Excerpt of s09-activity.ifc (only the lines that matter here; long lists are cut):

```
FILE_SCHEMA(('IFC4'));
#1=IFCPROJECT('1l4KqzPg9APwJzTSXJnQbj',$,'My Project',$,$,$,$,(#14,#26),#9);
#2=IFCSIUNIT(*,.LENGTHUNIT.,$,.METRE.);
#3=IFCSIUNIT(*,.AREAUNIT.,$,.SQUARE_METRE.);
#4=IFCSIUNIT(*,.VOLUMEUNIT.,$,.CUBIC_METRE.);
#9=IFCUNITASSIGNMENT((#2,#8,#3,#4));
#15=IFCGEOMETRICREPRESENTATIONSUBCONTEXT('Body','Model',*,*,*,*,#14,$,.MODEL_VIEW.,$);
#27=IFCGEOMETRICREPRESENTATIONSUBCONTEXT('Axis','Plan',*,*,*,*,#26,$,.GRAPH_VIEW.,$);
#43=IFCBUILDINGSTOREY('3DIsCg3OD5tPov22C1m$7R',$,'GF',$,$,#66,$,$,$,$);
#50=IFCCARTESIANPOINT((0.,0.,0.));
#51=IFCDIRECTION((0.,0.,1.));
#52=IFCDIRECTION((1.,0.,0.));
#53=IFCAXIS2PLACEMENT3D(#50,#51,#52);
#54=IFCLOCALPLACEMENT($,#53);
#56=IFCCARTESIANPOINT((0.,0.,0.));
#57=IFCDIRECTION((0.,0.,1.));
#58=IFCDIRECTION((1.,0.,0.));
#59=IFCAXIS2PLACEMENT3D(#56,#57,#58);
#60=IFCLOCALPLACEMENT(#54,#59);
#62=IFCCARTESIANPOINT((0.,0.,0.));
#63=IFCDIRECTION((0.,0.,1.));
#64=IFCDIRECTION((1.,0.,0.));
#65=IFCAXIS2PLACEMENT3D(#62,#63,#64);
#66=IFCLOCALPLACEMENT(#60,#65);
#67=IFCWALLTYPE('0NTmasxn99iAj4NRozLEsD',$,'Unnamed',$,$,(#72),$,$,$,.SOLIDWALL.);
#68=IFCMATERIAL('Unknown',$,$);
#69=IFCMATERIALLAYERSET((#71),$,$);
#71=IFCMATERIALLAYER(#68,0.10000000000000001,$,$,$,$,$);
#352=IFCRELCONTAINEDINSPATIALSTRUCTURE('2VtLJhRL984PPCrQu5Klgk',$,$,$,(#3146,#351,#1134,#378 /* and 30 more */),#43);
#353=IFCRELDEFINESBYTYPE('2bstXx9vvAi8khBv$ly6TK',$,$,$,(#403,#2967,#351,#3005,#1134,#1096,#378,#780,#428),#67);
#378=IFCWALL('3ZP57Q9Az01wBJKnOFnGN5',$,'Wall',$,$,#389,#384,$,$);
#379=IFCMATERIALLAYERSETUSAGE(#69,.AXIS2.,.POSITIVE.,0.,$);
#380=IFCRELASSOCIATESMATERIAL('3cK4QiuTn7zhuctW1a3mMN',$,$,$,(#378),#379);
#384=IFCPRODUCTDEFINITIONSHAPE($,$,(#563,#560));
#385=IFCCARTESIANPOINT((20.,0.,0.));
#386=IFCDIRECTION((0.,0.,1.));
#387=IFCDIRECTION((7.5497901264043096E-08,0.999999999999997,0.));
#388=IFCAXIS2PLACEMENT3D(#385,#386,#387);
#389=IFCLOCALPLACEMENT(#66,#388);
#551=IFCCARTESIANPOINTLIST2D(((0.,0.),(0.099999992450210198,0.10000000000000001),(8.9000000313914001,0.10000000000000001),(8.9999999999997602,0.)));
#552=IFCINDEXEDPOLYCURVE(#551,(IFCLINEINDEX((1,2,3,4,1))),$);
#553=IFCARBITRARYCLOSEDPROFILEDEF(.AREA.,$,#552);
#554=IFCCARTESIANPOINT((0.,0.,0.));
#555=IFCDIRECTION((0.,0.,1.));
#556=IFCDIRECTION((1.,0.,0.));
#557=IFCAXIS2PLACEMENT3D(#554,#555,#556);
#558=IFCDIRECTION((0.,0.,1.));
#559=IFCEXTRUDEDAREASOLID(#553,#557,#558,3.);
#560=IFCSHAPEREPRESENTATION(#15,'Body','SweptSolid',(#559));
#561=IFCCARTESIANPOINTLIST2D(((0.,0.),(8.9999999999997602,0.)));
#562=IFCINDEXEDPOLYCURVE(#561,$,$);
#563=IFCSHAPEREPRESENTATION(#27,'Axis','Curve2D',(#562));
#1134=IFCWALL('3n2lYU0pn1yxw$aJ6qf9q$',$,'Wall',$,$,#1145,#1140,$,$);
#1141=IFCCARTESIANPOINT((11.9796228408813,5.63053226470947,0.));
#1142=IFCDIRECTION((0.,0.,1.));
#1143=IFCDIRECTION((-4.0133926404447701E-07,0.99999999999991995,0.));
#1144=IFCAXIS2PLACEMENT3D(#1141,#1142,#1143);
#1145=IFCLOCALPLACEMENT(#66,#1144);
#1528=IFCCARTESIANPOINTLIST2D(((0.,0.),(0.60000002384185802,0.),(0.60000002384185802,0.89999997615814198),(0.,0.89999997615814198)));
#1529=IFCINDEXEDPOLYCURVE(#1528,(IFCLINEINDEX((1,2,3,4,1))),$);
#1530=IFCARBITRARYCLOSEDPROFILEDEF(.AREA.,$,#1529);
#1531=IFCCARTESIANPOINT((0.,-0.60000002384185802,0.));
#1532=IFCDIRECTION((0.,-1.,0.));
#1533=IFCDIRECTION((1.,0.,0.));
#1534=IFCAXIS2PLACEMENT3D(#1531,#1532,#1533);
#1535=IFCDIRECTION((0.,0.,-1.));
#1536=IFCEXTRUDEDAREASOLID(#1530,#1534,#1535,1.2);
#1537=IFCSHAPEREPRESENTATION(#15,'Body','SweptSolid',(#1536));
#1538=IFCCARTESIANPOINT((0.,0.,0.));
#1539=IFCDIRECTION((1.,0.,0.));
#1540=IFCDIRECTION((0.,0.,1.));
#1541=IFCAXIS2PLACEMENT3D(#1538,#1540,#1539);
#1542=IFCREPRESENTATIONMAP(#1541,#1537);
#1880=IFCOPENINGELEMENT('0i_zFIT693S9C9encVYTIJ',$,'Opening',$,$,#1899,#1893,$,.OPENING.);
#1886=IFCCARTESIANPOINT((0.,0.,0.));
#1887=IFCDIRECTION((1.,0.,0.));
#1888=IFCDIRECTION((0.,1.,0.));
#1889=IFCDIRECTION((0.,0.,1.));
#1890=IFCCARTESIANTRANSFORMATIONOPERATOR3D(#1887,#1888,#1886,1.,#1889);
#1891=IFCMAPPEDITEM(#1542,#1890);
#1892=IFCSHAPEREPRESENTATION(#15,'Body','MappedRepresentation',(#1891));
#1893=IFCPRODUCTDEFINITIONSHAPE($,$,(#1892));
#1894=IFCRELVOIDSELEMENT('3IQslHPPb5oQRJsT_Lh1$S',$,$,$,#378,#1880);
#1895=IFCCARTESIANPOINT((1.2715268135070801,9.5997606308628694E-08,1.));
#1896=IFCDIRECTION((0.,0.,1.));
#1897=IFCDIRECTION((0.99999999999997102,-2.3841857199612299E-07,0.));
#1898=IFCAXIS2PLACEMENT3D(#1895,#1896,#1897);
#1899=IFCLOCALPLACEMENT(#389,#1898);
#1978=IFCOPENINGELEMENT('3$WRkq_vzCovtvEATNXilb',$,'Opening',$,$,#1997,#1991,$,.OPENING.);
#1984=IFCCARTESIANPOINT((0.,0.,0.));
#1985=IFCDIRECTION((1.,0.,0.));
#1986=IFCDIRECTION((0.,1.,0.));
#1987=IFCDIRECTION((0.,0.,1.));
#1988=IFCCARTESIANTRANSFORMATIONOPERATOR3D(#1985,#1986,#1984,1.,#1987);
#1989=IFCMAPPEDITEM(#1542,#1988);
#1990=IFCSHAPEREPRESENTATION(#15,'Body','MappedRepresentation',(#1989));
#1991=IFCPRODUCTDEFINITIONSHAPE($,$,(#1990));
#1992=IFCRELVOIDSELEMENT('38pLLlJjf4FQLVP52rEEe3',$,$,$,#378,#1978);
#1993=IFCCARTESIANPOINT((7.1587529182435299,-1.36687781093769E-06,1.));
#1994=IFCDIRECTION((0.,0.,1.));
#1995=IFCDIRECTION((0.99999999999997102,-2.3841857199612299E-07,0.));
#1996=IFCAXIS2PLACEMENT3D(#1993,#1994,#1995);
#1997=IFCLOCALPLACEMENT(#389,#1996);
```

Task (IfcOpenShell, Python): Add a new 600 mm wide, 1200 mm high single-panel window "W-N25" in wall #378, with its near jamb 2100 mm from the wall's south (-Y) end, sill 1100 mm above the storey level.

```python
import numpy as np
import ifcopenshell
import ifcopenshell.api.feature
import ifcopenshell.api.geometry
import ifcopenshell.api.root
import ifcopenshell.api.spatial
import ifcopenshell.geom
import ifcopenshell.util.element
import ifcopenshell.util.placement
import ifcopenshell.util.representation
import ifcopenshell.util.shape
import ifcopenshell.util.unit

model = ifcopenshell.open("s09-activity.ifc")
unit_scale = ifcopenshell.util.unit.calculate_unit_scale(model)
settings = ifcopenshell.geom.settings()


def volume(element):
    """Net volume in cubic metres, openings subtracted."""
    shape = ifcopenshell.geom.create_shape(settings, element)
    return ifcopenshell.util.shape.get_volume(shape.geometry)


wall = model.by_guid("3ZP57Q9Az01wBJKnOFnGN5")
storey = ifcopenshell.util.element.get_container(wall, ifc_class="IfcBuildingStorey")
context = ifcopenshell.util.representation.get_context(model, "Model", "Body", "MODEL_VIEW")
before = volume(wall)

width, height, from_end, sill = 0.6, 1.2, 2.1, 1.1  # metres

# The wall runs along its own X axis, and the end named is its -X end.
wall_shape = ifcopenshell.geom.create_shape(settings, wall)
x, y, z = ifcopenshell.util.shape.get_vertices(wall_shape.geometry).T
start = x.min() + from_end
face, thickness = float(y.min()), float(y.max() - y.min())
wall_matrix = ifcopenshell.util.placement.get_local_placement(wall.ObjectPlacement)
level = ifcopenshell.util.placement.get_local_placement(storey.ObjectPlacement)[2, 3]


def in_wall(x, y):
    """Placement at x, y metres in the wall's axes, at sill height."""
    matrix = wall_matrix.copy()
    matrix[:, 3] = wall_matrix @ np.array([x / unit_scale, y / unit_scale, 0.0, 1.0])
    matrix[2, 3] = level + sill / unit_scale
    return matrix


# Opening: a box that overshoots both wall faces by 50 mm.
opening = ifcopenshell.api.root.create_entity(model, ifc_class="IfcOpeningElement", predefined_type="OPENING")
box = ifcopenshell.api.geometry.add_wall_representation(
    model, context=context, length=width, height=height, thickness=thickness + 0.1
)
ifcopenshell.api.geometry.assign_representation(model, product=opening, representation=box)
ifcopenshell.api.geometry.edit_object_placement(model, product=opening, matrix=in_wall(start, face - 0.05), is_si=False)
ifcopenshell.api.feature.add_feature(model, feature=opening, element=wall)

window = ifcopenshell.api.root.create_entity(model, ifc_class="IfcWindow", name="W-N25", predefined_type="WINDOW")
window.OverallWidth, window.OverallHeight = width / unit_scale, height / unit_scale
window.PartitioningType = "SINGLE_PANEL"
body = ifcopenshell.api.geometry.add_window_representation(
    model,
    context=context,
    overall_width=window.OverallWidth,
    overall_height=window.OverallHeight,
    partition_type="SINGLE_PANEL",
)
ifcopenshell.api.geometry.assign_representation(model, product=window, representation=body)
ifcopenshell.api.spatial.assign_container(model, products=[window], relating_structure=storey)
ifcopenshell.api.feature.add_filling(model, opening=opening, element=window)

# Centre the window in the wall's thickness.
ifcopenshell.api.geometry.edit_object_placement(model, product=window, matrix=in_wall(start, face), is_si=False)
window_shape = ifcopenshell.geom.create_shape(settings, window)
depth = ifcopenshell.util.shape.get_vertices(window_shape.geometry)[:, 1]
offset = face + thickness / 2 - (depth.min() + depth.max()) / 2
ifcopenshell.api.geometry.edit_object_placement(model, product=window, matrix=in_wall(start, offset), is_si=False)

after = volume(wall)

print(f"wall volume {before:.3f} -> {after:.3f} m3")

model.write("s09-activity_rev.ifc")
```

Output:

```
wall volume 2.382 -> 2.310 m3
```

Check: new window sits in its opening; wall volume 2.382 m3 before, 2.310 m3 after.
